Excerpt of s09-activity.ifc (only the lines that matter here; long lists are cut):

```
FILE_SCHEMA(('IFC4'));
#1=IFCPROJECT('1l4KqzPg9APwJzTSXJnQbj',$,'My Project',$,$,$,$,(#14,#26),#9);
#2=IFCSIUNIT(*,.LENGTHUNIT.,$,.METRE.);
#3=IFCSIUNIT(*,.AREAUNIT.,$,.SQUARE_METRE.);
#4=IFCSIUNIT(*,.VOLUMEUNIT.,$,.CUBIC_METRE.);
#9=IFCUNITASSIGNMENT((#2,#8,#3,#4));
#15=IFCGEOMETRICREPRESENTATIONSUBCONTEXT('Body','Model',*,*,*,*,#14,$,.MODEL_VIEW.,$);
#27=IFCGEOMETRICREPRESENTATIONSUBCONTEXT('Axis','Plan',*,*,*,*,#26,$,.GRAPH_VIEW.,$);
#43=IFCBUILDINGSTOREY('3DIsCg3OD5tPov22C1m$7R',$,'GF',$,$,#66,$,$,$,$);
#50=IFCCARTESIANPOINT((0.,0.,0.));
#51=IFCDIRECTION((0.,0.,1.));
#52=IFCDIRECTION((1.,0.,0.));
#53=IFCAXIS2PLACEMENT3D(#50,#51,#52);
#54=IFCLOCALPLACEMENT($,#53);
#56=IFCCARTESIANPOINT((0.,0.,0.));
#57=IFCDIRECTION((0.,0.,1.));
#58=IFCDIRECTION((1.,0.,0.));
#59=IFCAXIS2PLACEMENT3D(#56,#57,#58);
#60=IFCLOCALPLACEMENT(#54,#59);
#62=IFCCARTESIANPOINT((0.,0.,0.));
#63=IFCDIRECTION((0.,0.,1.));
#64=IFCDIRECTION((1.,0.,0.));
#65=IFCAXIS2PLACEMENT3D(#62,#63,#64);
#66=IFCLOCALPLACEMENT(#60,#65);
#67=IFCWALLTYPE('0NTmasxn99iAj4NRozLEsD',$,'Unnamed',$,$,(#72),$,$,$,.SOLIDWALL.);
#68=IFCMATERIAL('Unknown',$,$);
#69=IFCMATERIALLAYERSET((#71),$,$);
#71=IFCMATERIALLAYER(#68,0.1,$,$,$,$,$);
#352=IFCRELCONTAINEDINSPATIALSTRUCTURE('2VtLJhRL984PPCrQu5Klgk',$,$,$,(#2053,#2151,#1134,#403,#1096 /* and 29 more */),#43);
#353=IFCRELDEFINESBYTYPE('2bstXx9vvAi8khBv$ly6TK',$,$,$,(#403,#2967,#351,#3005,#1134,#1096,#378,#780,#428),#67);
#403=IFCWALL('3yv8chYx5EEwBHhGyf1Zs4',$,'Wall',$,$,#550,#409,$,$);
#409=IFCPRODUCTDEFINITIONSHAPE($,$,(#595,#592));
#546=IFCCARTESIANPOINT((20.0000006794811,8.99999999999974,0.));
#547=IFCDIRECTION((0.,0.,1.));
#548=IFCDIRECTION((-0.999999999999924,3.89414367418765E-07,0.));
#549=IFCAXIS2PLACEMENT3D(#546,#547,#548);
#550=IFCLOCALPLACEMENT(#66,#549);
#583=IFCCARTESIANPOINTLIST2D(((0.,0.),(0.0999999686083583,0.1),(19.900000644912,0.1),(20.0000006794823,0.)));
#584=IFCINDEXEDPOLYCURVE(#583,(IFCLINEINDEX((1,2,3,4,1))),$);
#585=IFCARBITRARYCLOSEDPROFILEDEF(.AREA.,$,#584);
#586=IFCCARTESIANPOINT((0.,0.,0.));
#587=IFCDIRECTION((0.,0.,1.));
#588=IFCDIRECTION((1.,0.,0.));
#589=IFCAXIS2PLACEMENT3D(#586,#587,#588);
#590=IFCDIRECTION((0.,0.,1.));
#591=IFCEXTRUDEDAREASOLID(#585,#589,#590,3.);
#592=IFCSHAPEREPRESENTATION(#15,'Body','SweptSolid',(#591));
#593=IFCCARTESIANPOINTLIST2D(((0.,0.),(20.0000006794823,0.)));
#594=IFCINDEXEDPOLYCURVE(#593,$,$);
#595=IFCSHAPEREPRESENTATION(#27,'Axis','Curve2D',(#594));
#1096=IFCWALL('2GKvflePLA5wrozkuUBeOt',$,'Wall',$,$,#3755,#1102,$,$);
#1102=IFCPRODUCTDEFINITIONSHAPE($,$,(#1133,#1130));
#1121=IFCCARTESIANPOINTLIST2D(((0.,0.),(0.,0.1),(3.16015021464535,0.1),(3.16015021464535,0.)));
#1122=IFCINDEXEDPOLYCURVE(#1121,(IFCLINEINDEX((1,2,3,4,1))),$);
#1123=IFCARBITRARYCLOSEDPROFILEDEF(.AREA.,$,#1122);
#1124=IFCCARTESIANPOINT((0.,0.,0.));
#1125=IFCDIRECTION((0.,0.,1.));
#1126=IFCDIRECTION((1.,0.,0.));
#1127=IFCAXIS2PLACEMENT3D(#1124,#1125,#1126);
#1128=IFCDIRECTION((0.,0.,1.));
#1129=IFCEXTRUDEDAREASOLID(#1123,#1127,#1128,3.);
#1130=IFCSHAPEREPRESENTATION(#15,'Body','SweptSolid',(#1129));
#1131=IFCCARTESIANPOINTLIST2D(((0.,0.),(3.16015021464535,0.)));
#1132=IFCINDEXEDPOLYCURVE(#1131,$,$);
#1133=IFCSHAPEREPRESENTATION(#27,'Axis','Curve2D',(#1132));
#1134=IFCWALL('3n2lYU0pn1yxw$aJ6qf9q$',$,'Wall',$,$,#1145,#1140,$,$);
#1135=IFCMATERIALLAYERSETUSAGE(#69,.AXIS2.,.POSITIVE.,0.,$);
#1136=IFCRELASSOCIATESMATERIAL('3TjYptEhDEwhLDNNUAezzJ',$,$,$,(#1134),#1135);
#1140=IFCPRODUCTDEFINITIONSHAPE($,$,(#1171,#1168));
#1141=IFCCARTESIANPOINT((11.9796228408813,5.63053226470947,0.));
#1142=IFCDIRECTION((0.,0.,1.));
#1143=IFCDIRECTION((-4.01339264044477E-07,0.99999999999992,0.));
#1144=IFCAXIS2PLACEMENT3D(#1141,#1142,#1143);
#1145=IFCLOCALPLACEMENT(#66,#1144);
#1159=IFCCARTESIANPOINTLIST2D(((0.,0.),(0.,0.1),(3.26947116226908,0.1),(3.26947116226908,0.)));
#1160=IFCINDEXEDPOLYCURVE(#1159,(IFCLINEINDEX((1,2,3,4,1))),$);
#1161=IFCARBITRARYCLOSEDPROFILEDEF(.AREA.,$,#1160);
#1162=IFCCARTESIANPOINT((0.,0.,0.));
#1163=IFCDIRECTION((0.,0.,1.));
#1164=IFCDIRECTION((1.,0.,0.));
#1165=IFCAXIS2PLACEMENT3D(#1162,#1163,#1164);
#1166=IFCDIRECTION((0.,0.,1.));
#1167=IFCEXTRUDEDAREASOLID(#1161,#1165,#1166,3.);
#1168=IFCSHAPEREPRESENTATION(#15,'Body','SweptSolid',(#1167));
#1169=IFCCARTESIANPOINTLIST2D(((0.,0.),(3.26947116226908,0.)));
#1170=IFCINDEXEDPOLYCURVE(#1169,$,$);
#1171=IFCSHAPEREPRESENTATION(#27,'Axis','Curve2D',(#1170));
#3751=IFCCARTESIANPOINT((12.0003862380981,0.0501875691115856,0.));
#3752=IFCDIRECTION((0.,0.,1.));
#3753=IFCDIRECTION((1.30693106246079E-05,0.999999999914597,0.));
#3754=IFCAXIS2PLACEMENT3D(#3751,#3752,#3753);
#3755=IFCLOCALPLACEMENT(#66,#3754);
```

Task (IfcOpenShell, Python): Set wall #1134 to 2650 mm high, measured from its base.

```python
import ifcopenshell
import ifcopenshell.geom
import ifcopenshell.util.representation
import ifcopenshell.util.shape

model = ifcopenshell.open("s09-activity.ifc")
settings = ifcopenshell.geom.settings()


def volume(element):
    """Net volume in cubic metres, openings subtracted."""
    shape = ifcopenshell.geom.create_shape(settings, element)
    return ifcopenshell.util.shape.get_volume(shape.geometry)


wall = model.by_guid("3n2lYU0pn1yxw$aJ6qf9q$")
before = volume(wall)

body = ifcopenshell.util.representation.get_representation(wall, "Model", "Body")
solid = body.Items[0]
old_height = solid.Depth
solid.Depth = 2.65
after = volume(wall)

print(f"height {old_height:g} -> {solid.Depth:g}, volume {before:.3f} -> {after:.3f} m3")

model.write("s09-activity-out.ifc")
```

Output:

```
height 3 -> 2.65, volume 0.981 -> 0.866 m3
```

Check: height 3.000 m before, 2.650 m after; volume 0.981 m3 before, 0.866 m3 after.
